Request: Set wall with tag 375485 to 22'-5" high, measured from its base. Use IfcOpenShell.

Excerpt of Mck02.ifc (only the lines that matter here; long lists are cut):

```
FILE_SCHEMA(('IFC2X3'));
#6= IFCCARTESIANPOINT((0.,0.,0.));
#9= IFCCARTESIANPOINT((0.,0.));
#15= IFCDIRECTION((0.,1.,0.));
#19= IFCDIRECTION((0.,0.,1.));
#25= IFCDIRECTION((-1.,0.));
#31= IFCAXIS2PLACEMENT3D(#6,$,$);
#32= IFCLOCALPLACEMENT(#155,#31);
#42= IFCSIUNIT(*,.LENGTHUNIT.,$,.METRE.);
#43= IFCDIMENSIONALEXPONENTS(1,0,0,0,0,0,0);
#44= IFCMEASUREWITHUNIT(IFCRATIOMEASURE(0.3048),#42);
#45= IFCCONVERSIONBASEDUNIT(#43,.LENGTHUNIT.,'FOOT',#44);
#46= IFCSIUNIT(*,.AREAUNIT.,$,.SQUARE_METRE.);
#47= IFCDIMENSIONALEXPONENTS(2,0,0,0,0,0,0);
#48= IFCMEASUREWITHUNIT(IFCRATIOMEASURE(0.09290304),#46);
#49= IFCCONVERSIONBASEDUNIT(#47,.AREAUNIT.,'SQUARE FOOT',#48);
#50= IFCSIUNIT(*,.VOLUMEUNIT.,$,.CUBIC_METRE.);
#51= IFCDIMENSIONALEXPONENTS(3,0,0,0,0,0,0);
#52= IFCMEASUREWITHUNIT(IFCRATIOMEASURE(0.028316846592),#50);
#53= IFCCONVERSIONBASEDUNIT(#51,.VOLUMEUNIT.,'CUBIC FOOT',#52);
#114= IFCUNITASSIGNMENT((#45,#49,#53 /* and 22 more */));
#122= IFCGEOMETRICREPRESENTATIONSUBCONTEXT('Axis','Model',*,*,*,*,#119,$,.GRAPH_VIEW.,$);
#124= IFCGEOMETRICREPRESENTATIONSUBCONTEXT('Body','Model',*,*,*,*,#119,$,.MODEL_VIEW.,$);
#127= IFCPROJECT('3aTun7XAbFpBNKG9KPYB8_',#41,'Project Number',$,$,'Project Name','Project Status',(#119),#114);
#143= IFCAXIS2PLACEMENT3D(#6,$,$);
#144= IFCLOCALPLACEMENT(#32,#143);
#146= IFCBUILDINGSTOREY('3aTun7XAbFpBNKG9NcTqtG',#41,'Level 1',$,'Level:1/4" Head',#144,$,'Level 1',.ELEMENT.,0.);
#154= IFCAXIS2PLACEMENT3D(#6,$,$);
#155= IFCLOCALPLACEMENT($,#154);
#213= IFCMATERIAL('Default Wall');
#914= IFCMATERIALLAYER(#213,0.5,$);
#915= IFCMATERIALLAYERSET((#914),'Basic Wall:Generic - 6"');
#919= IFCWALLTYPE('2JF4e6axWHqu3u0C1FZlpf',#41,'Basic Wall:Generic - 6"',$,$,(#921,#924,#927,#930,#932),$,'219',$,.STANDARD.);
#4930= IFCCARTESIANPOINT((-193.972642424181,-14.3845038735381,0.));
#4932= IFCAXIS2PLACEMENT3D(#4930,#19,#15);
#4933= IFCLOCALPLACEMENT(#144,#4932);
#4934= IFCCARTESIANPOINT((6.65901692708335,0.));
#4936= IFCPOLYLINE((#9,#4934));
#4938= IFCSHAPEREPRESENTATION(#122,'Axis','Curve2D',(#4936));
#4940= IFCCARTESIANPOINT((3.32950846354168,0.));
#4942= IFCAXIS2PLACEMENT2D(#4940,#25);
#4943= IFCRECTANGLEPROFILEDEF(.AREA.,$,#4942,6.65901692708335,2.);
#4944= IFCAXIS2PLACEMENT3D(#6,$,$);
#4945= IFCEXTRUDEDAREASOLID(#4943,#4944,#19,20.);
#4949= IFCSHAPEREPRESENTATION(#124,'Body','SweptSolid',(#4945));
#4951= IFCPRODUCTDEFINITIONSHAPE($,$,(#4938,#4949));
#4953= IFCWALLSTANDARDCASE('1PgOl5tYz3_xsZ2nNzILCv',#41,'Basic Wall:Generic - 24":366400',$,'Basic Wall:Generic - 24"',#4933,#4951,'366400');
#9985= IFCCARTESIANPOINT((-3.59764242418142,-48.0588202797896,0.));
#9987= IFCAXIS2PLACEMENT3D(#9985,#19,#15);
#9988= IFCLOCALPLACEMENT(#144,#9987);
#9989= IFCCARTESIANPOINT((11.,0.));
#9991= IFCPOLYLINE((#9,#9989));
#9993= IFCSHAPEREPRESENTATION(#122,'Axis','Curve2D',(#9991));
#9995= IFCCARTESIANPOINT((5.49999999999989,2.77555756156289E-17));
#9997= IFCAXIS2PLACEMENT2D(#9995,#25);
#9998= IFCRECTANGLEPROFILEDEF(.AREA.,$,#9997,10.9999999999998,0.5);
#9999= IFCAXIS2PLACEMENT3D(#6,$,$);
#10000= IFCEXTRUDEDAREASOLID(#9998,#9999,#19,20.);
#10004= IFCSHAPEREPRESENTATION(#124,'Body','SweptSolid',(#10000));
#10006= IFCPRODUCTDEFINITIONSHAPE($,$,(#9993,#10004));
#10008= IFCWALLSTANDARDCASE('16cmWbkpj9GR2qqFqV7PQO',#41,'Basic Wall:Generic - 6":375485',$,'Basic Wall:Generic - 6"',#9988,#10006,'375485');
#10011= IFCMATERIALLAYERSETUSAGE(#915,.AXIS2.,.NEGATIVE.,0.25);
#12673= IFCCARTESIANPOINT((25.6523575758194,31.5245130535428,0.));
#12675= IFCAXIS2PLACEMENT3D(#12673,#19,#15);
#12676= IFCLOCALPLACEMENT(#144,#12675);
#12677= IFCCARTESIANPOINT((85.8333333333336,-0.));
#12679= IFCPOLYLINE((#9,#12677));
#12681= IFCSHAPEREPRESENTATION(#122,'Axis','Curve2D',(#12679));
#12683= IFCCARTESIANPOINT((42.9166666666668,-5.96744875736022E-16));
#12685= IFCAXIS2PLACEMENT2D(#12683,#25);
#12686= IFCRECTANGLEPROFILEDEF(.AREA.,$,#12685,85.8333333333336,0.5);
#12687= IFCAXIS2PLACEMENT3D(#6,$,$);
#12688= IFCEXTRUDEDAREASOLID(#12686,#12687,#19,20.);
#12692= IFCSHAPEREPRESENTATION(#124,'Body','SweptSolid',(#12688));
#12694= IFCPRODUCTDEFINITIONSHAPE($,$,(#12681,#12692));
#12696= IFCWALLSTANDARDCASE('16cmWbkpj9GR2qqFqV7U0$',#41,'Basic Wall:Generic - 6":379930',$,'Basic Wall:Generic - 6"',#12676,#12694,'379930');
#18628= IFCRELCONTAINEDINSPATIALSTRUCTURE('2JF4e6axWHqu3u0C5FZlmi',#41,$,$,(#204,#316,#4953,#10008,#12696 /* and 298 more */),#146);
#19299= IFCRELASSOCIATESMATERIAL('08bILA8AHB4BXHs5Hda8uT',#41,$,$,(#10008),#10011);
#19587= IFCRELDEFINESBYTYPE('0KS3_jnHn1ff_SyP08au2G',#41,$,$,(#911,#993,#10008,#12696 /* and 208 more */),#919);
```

```python
import ifcopenshell
import ifcopenshell.geom
import ifcopenshell.util.representation
import ifcopenshell.util.shape
import ifcopenshell.util.unit

model = ifcopenshell.open("Mck02.ifc")
unit_scale = ifcopenshell.util.unit.calculate_unit_scale(model)
settings = ifcopenshell.geom.settings()


def volume(element):
    """Net volume in cubic metres, openings subtracted."""
    shape = ifcopenshell.geom.create_shape(settings, element)
    return ifcopenshell.util.shape.get_volume(shape.geometry)


wall = model.by_id(10008)
before = volume(wall)

body = ifcopenshell.util.representation.get_representation(wall, "Model", "Body")
solid = body.Items[0]
old_height = solid.Depth
solid.Depth = 269 * 0.0254 / unit_scale
after = volume(wall)

print(f"height {old_height:g} -> {solid.Depth:g}, volume {before:.3f} -> {after:.3f} m3")

model.write("Mck02_edited.ifc")
```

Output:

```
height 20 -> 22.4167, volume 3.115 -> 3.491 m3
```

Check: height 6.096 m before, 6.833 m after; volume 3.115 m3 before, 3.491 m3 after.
